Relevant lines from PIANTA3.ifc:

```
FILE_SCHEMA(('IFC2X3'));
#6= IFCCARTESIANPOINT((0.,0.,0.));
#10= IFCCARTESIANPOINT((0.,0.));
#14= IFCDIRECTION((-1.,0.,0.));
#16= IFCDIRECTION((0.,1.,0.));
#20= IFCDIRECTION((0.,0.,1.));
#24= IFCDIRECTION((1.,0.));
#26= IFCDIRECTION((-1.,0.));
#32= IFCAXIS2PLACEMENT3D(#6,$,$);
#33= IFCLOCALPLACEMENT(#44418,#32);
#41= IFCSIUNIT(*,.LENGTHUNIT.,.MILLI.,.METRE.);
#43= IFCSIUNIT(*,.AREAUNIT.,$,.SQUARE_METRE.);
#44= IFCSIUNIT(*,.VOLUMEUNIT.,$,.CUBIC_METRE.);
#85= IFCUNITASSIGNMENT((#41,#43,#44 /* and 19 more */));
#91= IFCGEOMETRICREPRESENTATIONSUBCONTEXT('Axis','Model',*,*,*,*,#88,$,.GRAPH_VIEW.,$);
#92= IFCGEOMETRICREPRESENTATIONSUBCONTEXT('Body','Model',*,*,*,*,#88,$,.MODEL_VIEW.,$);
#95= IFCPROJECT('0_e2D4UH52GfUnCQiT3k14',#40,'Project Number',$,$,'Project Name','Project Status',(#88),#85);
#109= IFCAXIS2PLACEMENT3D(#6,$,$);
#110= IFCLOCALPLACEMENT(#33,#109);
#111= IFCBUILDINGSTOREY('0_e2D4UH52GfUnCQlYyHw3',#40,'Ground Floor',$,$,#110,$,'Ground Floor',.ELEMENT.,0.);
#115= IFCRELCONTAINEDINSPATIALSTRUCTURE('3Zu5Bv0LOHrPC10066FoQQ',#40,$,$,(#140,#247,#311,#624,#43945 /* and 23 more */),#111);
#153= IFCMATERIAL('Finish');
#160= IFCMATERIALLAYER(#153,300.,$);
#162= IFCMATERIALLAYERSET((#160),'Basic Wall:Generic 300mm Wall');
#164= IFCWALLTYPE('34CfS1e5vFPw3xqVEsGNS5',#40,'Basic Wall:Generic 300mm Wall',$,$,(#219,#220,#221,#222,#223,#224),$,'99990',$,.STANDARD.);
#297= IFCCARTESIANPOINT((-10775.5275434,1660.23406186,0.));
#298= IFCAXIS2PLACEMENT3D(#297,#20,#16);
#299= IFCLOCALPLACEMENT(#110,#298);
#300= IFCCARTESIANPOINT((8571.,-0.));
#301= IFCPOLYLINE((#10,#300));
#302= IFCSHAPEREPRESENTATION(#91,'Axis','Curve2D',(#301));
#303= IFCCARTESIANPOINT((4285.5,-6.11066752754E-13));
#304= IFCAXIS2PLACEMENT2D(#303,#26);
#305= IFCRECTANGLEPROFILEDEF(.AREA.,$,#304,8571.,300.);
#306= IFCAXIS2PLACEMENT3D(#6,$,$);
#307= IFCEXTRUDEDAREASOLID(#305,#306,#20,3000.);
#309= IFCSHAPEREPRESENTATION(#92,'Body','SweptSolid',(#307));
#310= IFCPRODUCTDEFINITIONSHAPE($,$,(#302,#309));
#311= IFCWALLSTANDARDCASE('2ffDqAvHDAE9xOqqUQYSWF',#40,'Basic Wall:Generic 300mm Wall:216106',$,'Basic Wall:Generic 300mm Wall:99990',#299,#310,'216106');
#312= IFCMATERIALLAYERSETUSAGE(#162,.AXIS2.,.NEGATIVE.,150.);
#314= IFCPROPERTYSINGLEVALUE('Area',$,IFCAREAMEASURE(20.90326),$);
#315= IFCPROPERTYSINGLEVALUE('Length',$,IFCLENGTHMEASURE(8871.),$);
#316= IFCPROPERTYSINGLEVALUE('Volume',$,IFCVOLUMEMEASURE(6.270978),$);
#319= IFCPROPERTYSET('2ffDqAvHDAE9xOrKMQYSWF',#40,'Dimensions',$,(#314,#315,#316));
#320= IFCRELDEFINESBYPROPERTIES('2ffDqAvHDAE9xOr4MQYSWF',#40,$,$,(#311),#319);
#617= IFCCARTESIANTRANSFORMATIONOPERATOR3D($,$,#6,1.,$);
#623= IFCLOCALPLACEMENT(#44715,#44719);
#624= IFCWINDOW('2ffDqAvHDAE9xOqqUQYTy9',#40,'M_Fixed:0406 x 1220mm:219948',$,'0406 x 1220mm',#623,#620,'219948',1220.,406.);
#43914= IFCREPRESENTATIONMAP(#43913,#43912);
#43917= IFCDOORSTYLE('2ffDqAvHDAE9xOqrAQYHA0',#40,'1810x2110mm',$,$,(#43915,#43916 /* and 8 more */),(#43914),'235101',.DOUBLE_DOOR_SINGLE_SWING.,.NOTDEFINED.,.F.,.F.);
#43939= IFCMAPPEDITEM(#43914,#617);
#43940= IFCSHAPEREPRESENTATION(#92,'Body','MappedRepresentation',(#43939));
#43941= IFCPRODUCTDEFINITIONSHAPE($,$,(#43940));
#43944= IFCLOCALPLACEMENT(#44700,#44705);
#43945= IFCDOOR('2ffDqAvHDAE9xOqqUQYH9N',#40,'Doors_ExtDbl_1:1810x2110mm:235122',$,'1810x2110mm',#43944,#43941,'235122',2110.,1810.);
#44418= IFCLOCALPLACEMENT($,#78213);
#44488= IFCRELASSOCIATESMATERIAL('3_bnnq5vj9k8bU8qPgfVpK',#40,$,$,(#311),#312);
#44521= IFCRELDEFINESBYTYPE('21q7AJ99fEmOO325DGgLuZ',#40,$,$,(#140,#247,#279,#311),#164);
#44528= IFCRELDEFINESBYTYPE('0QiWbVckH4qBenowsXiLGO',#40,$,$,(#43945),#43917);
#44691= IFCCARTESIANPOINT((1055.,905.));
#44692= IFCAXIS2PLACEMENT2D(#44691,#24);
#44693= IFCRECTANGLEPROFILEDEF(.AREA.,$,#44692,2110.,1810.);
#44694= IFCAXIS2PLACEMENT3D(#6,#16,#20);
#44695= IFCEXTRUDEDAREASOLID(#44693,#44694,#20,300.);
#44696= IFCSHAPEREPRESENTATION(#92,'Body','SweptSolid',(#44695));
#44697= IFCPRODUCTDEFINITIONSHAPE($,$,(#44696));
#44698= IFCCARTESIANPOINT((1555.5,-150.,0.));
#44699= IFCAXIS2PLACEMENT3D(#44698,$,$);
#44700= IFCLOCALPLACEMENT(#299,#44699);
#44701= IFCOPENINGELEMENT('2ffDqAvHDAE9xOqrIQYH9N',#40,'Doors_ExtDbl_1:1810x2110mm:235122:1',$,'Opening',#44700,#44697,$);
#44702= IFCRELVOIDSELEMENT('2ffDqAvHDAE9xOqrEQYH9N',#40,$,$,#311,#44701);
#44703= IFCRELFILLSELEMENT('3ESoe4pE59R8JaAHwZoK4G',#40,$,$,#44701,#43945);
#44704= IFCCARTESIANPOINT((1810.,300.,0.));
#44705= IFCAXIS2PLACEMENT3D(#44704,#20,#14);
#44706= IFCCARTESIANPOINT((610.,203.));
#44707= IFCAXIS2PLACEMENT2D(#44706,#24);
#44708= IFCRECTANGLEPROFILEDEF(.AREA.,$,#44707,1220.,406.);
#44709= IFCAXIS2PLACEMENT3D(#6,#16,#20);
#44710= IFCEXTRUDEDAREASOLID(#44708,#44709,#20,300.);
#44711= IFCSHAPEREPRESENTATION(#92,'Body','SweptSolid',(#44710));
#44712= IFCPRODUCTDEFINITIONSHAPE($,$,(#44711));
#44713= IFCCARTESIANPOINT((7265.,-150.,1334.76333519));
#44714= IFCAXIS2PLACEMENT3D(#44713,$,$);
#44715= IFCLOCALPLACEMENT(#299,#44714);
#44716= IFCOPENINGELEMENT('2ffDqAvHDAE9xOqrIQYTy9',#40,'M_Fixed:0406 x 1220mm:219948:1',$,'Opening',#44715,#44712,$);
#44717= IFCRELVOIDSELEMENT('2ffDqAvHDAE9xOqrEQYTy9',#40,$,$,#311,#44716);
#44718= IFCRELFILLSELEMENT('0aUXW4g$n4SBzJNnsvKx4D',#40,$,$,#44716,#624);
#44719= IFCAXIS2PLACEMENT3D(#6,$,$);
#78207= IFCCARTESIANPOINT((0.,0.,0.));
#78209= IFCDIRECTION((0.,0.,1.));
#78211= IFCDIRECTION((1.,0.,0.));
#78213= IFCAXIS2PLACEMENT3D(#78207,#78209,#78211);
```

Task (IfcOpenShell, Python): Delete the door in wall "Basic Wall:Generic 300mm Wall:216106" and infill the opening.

```python
import ifcopenshell
import ifcopenshell.api.feature
import ifcopenshell.api.pset
import ifcopenshell.api.root
import ifcopenshell.geom
import ifcopenshell.util.element
import ifcopenshell.util.shape
import ifcopenshell.util.unit

model = ifcopenshell.open("PIANTA3.ifc")
area_scale = ifcopenshell.util.unit.calculate_unit_scale(model, "AREAUNIT")
volume_scale = ifcopenshell.util.unit.calculate_unit_scale(model, "VOLUMEUNIT")
settings = ifcopenshell.geom.settings()


def volume(element):
    """Net volume in cubic metres, openings subtracted."""
    shape = ifcopenshell.geom.create_shape(settings, element)
    return ifcopenshell.util.shape.get_volume(shape.geometry)


door = model.by_guid("2ffDqAvHDAE9xOqqUQYH9N")
opening = door.FillsVoids[0].RelatingOpeningElement
wall = opening.VoidsElements[0].RelatingBuildingElement
before = volume(wall)

ifcopenshell.api.root.remove_product(model, product=door)
ifcopenshell.api.feature.remove_feature(model, feature=opening)

after = volume(wall)
thickness = 0.3  # wall thickness in metres

# Update the wall's stored quantities.
pset = model.by_id(ifcopenshell.util.element.get_pset(wall, "Dimensions", should_inherit=False)["id"])
ifcopenshell.api.pset.edit_pset(model, pset=pset, properties={
    "Area": model.create_entity("IfcAreaMeasure", after / thickness / area_scale),
    "Volume": model.create_entity("IfcVolumeMeasure", after / volume_scale),
})

print(f"wall volume {before:.3f} -> {after:.3f} m3")

model.write("PIANTA3-out.ifc")
```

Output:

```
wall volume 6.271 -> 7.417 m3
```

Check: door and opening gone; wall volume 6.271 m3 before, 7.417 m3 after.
